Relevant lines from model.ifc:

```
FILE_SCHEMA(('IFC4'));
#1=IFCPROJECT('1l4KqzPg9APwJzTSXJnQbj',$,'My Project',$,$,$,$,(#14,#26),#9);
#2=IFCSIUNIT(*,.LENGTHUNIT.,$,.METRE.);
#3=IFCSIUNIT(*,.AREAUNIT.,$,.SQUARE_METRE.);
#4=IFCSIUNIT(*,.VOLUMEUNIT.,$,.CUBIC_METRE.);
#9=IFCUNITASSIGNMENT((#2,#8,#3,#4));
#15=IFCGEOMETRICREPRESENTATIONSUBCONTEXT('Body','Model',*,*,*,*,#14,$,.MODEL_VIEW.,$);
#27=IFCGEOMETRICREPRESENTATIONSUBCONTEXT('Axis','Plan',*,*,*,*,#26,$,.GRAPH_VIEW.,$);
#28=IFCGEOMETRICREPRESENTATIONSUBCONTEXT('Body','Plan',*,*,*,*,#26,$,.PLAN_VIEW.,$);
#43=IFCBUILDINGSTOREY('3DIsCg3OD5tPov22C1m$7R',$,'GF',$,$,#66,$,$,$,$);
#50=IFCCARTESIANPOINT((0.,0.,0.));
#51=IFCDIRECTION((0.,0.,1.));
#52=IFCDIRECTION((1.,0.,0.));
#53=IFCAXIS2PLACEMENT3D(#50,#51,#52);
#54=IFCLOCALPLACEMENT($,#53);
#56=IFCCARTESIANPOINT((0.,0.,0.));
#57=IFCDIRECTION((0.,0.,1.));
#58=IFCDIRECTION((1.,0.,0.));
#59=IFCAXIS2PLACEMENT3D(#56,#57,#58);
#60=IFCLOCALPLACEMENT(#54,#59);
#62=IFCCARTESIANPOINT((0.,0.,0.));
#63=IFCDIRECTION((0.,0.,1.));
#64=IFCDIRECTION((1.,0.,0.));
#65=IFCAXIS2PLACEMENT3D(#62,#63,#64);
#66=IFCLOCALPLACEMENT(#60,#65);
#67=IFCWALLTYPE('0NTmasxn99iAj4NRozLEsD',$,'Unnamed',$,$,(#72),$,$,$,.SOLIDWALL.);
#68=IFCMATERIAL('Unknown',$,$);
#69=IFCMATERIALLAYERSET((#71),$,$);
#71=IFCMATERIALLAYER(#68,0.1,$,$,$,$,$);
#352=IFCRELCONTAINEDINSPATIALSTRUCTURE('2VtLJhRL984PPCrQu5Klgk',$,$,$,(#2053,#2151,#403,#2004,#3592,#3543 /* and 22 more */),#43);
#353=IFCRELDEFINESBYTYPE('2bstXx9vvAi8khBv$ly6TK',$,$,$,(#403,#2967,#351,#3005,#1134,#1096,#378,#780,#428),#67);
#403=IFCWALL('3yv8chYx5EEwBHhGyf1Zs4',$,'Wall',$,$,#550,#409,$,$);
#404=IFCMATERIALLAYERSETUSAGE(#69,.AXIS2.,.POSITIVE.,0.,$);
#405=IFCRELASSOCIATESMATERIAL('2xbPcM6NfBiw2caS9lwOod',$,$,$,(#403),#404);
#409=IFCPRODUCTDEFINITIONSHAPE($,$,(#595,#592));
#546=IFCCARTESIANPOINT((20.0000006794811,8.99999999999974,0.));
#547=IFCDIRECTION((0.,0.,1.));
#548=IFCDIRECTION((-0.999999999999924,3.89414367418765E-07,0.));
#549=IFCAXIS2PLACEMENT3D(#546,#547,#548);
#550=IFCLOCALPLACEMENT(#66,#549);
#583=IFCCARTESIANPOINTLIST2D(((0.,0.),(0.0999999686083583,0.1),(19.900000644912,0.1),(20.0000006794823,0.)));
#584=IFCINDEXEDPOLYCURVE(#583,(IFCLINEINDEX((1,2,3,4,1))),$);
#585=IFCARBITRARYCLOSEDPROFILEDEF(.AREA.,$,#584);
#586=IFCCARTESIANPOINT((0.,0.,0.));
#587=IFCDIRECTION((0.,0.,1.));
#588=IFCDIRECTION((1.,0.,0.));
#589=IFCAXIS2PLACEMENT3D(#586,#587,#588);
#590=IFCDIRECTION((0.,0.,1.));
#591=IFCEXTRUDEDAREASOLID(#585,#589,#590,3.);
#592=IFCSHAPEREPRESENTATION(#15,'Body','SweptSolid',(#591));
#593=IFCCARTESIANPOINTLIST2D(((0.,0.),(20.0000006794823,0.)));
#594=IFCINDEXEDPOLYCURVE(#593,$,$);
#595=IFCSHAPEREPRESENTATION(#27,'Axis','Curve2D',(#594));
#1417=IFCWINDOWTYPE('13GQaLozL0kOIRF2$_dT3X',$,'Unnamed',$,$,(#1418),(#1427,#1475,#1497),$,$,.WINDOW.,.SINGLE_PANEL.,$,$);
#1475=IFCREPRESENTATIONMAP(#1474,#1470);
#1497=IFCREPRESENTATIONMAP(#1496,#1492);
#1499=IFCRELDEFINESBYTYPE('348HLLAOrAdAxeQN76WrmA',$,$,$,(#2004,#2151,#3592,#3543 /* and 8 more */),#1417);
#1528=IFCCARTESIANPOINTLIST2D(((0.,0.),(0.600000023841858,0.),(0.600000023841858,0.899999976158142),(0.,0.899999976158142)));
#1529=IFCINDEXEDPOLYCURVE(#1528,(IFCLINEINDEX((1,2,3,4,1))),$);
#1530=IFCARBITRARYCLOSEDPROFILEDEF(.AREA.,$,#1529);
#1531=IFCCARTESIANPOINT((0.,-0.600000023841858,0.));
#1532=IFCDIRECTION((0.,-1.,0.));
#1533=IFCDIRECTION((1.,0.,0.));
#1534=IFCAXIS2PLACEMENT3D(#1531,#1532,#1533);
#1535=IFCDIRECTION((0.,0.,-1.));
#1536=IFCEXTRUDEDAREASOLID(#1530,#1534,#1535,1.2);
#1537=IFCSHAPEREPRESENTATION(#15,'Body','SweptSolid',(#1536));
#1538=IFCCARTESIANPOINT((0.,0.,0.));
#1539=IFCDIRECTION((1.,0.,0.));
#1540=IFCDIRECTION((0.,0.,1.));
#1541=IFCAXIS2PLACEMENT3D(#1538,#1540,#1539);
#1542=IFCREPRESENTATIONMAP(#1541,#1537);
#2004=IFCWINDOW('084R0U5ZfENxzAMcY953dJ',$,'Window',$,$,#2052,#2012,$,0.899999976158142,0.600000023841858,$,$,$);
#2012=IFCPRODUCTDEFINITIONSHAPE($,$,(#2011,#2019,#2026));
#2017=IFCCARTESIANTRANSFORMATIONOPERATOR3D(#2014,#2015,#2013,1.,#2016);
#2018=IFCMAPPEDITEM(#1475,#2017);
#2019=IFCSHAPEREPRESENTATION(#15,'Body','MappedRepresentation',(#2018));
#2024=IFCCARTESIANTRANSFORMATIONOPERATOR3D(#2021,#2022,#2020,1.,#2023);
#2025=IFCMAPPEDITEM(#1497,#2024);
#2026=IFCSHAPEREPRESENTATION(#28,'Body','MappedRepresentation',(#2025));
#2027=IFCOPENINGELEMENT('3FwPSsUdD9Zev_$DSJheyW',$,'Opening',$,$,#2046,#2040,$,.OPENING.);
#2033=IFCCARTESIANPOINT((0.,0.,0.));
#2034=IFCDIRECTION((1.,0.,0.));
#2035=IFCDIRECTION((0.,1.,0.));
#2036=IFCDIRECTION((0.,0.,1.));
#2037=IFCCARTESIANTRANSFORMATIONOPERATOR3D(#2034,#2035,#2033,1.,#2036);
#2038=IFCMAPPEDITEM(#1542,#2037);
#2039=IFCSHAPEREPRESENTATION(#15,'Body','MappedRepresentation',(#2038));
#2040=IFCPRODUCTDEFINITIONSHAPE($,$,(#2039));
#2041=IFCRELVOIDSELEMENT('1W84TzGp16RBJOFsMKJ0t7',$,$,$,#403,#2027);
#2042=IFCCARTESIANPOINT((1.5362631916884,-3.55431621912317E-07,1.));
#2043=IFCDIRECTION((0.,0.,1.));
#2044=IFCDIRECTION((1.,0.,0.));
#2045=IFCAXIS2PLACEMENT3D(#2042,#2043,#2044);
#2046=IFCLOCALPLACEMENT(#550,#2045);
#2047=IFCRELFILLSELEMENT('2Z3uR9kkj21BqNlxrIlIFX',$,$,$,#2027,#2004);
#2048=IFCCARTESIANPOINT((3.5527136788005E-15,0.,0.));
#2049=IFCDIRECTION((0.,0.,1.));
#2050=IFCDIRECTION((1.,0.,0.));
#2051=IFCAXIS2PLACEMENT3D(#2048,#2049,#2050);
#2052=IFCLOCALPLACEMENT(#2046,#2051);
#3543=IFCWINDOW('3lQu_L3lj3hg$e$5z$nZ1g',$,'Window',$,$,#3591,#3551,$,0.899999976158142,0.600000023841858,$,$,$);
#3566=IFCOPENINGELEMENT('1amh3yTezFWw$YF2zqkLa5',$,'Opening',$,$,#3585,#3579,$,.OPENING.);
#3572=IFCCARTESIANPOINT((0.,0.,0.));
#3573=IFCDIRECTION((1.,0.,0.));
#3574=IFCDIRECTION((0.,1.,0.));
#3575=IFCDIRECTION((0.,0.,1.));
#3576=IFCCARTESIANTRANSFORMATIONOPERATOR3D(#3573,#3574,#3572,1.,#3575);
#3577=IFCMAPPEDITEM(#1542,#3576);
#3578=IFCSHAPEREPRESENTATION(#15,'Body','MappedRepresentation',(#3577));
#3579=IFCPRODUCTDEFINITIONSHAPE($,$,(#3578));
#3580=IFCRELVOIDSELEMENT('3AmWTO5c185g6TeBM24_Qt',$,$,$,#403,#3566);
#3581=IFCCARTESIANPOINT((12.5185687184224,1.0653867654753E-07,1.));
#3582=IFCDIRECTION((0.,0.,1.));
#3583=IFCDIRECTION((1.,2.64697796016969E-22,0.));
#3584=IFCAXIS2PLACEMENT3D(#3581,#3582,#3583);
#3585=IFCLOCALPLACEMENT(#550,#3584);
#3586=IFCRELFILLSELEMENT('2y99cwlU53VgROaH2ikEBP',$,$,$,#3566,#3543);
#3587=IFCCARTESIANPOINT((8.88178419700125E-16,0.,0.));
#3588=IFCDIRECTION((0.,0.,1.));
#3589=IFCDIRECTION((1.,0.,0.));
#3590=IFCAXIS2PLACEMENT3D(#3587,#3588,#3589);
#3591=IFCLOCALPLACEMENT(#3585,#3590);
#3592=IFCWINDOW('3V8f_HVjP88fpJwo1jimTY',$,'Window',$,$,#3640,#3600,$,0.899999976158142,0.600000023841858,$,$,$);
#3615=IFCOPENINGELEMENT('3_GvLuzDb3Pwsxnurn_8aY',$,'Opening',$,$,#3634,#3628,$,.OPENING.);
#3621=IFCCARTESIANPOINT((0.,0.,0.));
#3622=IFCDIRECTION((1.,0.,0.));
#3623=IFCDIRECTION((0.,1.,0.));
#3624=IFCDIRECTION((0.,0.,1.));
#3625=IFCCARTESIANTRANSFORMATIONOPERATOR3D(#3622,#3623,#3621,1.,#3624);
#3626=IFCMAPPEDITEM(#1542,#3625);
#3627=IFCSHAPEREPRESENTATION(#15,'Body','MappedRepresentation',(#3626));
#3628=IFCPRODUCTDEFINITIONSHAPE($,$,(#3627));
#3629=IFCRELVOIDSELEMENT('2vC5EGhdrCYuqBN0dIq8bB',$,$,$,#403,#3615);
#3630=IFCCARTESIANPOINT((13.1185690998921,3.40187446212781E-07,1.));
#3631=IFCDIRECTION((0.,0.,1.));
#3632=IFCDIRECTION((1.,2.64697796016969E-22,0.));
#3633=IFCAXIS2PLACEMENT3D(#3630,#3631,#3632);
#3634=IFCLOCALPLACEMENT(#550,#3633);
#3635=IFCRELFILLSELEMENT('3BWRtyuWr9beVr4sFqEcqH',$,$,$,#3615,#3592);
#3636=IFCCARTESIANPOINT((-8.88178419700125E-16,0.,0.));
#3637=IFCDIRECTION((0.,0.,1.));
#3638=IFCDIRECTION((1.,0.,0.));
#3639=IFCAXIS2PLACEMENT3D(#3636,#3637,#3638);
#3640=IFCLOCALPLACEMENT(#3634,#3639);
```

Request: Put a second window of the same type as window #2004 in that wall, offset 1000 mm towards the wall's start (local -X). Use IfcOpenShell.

```python
import ifcopenshell
import ifcopenshell.api.feature
import ifcopenshell.api.geometry
import ifcopenshell.api.root
import ifcopenshell.geom
import ifcopenshell.util.element
import ifcopenshell.util.placement
import ifcopenshell.util.shape

model = ifcopenshell.open("model.ifc")
settings = ifcopenshell.geom.settings()


def volume(element):
    """Net volume in cubic metres, openings subtracted."""
    shape = ifcopenshell.geom.create_shape(settings, element)
    return ifcopenshell.util.shape.get_volume(shape.geometry)


window = model.by_guid("084R0U5ZfENxzAMcY953dJ")
opening = window.FillsVoids[0].RelatingOpeningElement
wall = opening.VoidsElements[0].RelatingBuildingElement
before = volume(wall)
shift = ifcopenshell.util.placement.get_local_placement(wall.ObjectPlacement)[:3, 0] * -1.0

# copy_class copies the void relationship, type, container and properties, but no geometry.
new_opening = ifcopenshell.api.root.copy_class(model, product=opening)
new_opening.Representation = ifcopenshell.util.element.copy_deep(
    model, opening.Representation, exclude=["IfcGeometricRepresentationContext", "IfcRepresentationMap"]
)
new_window = ifcopenshell.api.root.copy_class(model, product=window)
new_window.Representation = ifcopenshell.util.element.copy_deep(
    model, window.Representation, exclude=["IfcGeometricRepresentationContext", "IfcRepresentationMap"]
)
ifcopenshell.api.feature.add_filling(model, opening=new_opening, element=new_window)

for old, new in ((opening, new_opening), (window, new_window)):
    matrix = ifcopenshell.util.placement.get_local_placement(old.ObjectPlacement)
    matrix[:3, 3] += shift
    ifcopenshell.api.geometry.edit_object_placement(model, product=new, matrix=matrix, is_si=False)

after = volume(wall)

print(f"wall volume {before:.3f} -> {after:.3f} m3")

model.write("model_v2.ifc")
```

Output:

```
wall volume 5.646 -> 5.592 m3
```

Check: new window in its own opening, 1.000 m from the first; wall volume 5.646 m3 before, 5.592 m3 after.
